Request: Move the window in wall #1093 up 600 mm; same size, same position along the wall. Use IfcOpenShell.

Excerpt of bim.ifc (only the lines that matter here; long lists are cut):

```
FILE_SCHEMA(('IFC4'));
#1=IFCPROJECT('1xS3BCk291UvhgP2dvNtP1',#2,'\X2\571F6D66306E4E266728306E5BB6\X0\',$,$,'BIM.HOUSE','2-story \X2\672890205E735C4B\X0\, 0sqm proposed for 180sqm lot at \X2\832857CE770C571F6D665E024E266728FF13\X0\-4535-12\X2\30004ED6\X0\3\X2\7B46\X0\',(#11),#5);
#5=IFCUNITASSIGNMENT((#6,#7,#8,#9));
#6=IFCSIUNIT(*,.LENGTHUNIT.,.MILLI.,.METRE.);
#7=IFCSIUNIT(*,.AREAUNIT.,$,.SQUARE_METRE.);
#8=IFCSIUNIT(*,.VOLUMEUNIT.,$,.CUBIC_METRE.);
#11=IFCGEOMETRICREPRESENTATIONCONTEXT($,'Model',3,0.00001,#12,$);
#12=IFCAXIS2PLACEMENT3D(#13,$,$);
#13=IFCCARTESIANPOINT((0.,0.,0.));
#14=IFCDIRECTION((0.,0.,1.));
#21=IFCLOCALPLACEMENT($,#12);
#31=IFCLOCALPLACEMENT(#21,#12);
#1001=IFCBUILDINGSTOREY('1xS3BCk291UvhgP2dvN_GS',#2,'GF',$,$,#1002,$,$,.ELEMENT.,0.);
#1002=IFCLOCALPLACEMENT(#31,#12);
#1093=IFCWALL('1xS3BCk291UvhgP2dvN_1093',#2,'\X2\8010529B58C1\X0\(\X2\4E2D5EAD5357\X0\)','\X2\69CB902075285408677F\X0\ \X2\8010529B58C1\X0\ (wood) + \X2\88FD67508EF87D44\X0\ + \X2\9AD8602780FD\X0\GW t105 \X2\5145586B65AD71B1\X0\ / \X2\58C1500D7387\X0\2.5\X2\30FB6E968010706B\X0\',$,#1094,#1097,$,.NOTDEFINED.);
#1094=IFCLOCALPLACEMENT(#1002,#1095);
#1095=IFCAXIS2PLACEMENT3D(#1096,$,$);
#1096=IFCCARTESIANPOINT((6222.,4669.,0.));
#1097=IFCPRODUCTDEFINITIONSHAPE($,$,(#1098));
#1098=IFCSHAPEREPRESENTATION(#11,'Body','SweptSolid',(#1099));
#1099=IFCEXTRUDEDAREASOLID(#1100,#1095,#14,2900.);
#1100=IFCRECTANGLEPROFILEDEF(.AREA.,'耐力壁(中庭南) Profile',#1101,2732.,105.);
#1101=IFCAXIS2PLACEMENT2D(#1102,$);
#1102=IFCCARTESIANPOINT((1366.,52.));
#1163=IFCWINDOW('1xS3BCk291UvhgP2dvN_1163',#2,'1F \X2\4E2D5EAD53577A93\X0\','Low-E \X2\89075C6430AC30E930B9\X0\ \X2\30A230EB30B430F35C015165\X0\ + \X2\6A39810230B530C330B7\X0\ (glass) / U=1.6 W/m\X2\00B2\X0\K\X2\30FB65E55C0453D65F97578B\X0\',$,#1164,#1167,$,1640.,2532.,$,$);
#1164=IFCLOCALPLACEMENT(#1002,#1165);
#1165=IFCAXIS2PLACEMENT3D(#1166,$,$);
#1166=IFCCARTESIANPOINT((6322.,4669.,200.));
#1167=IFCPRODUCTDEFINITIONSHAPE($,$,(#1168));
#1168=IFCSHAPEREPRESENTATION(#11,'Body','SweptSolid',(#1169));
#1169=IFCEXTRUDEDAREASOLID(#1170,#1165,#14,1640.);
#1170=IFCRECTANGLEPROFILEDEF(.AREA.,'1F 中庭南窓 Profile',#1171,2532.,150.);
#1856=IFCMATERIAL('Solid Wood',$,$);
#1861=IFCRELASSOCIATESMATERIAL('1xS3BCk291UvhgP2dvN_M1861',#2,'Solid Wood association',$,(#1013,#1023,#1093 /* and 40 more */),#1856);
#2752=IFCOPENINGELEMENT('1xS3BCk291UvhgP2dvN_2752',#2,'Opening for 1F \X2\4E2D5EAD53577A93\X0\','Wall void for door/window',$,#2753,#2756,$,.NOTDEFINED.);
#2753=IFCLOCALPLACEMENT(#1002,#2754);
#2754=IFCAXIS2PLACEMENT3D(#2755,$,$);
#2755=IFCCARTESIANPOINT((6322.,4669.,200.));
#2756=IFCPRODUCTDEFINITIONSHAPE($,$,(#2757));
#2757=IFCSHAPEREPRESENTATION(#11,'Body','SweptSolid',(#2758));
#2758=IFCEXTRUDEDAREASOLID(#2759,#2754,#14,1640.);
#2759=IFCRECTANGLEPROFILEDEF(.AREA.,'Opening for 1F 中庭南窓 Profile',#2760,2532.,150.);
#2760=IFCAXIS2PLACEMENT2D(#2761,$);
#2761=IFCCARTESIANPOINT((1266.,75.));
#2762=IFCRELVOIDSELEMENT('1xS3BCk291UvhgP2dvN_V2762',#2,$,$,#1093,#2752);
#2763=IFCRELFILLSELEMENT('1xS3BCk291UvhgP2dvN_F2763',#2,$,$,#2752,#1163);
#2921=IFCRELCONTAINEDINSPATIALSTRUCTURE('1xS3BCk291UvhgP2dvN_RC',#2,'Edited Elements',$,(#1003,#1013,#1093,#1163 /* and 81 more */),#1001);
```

```python
import numpy as np
import ifcopenshell
import ifcopenshell.api.geometry
import ifcopenshell.util.placement
import ifcopenshell.util.unit

model = ifcopenshell.open("bim.ifc")
unit_scale = ifcopenshell.util.unit.calculate_unit_scale(model)

window = model.by_guid("1xS3BCk291UvhgP2dvN_1163")
opening = window.FillsVoids[0].RelatingOpeningElement
dz = 0.6 / unit_scale

shift = np.array([0.0, 0.0, dz])
# The window is not placed relative to its opening, so move both.
for product in (opening, window):
    matrix = ifcopenshell.util.placement.get_local_placement(product.ObjectPlacement)
    matrix[:3, 3] += shift
    ifcopenshell.api.geometry.edit_object_placement(model, product=product, matrix=matrix, is_si=False)

print(f"moved by {dz * unit_scale:+.3f} m")

model.write("bim-out.ifc")
```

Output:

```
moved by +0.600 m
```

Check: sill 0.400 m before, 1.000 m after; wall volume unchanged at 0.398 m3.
